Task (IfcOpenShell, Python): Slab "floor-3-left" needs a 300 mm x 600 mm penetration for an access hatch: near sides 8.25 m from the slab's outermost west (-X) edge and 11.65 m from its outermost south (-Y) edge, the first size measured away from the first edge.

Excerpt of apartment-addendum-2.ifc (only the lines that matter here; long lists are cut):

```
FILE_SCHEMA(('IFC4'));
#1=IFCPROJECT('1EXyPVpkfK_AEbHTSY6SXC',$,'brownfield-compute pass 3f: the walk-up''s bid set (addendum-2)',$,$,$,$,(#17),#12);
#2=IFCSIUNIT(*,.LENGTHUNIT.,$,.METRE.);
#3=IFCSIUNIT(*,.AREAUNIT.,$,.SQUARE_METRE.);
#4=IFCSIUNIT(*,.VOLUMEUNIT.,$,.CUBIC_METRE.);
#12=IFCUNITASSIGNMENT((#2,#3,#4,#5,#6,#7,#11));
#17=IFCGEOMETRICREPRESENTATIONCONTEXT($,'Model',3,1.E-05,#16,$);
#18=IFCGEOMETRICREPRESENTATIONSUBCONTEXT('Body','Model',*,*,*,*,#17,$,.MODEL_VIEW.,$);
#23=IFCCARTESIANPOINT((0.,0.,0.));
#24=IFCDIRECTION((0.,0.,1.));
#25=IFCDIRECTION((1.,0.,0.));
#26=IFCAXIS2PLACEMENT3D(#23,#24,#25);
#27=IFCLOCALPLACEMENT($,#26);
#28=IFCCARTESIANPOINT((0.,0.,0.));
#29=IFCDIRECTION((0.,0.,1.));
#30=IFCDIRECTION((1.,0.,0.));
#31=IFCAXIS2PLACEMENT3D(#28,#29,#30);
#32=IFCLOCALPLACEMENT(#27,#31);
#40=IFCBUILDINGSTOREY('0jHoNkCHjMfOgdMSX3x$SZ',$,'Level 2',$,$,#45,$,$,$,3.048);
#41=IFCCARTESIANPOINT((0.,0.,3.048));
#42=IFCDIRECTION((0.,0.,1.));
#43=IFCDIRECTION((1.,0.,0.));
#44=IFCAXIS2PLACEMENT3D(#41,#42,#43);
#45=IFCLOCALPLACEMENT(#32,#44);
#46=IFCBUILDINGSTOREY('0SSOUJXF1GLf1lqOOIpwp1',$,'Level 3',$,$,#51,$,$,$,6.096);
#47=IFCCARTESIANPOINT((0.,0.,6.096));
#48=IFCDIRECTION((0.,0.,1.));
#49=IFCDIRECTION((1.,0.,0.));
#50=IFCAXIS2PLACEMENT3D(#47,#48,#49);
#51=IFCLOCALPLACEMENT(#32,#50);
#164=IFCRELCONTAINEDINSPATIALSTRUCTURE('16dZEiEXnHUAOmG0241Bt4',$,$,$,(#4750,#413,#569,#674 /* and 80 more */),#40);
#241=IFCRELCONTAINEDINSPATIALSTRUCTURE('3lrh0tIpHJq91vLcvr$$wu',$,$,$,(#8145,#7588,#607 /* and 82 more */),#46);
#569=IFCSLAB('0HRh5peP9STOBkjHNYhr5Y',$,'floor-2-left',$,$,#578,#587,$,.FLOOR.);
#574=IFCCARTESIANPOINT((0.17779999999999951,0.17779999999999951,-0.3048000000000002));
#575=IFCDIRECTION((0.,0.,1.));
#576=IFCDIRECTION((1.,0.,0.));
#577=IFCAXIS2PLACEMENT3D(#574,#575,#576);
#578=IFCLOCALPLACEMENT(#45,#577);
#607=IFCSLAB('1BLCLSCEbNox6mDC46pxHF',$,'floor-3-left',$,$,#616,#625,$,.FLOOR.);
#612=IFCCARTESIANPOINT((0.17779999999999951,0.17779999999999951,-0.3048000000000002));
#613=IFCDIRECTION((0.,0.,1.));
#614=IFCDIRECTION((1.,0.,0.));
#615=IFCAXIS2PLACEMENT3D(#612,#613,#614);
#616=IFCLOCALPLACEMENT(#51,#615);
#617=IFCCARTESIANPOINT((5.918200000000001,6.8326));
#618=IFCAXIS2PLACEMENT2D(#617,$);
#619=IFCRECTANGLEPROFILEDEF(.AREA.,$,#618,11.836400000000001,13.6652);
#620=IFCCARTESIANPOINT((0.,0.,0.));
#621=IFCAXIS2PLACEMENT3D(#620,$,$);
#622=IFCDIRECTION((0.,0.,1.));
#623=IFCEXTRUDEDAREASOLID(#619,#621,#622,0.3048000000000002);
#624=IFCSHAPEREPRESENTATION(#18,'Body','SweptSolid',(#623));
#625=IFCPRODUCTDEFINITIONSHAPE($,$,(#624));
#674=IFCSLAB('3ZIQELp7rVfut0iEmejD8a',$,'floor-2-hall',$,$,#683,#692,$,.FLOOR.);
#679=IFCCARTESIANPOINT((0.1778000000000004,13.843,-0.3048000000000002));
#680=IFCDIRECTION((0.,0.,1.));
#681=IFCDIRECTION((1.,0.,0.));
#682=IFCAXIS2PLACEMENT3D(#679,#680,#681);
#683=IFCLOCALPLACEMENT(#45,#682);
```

```python
import numpy as np
import ifcopenshell
import ifcopenshell.api.feature
import ifcopenshell.api.geometry
import ifcopenshell.api.root
import ifcopenshell.geom
import ifcopenshell.util.placement
import ifcopenshell.util.representation
import ifcopenshell.util.shape
import ifcopenshell.util.unit

model = ifcopenshell.open("apartment-addendum-2.ifc")
unit_scale = ifcopenshell.util.unit.calculate_unit_scale(model)
settings = ifcopenshell.geom.settings()


def volume(element):
    """Net volume in cubic metres, openings subtracted."""
    shape = ifcopenshell.geom.create_shape(settings, element)
    return ifcopenshell.util.shape.get_volume(shape.geometry)


slab = model.by_id(607)
before = volume(slab)

# Extent in the slab's own axes, in metres. The edges named are its -X and -Y sides.
slab_shape = ifcopenshell.geom.create_shape(settings, slab)
vertices = ifcopenshell.util.shape.get_vertices(slab_shape.geometry)
x_min, y_min, bottom = vertices.min(axis=0)
top = vertices[:, 2].max()

opening = ifcopenshell.api.root.create_entity(model, ifc_class="IfcOpeningElement", name="Access hatch opening", predefined_type="OPENING")
context = ifcopenshell.util.representation.get_context(model, "Model", "Body", "MODEL_VIEW")
width, depth = 0.3, 0.6
outline = [(0.0, 0.0), (width, 0.0), (width, depth), (0.0, depth), (0.0, 0.0)]
# Overshoot both faces by 50 mm so the cut is clean.
shape = ifcopenshell.api.geometry.add_slab_representation(
    model, context=context, depth=top - bottom + 0.1, polyline=outline
)
ifcopenshell.api.geometry.assign_representation(model, product=opening, representation=shape)

matrix = ifcopenshell.util.placement.get_local_placement(slab.ObjectPlacement)
matrix[:, 3] = matrix @ np.append(np.array([x_min + 8.25, y_min + 11.65, bottom - 0.05]) / unit_scale, 1.0)
ifcopenshell.api.geometry.edit_object_placement(model, product=opening, matrix=matrix, is_si=False)
ifcopenshell.api.feature.add_feature(model, feature=opening, element=slab)

after = volume(slab)

print(f"slab volume {before:.3f} -> {after:.3f} m3")

model.write("apartment-addendum-2_v2.ifc")
```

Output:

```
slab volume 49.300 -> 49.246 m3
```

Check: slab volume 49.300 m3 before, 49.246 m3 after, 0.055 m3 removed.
